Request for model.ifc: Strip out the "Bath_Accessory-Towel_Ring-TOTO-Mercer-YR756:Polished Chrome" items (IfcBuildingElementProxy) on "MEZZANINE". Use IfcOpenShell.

First a look at what the model holds.

```python
import ifcopenshell
import ifcopenshell.util.element

model = ifcopenshell.open("model.ifc")
print(model.schema)
storey = next(s for s in model.by_type("IfcBuildingStorey") if s.Name == "MEZZANINE")
proxies = [e for e in ifcopenshell.util.element.get_decomposition(storey) if e.is_a("IfcBuildingElementProxy")]
seen = {}
for e in proxies:
    element_type = ifcopenshell.util.element.get_type(e)
    name = element_type.Name if element_type not in (None, e) else None
    seen[name] = seen.get(name, 0) + 1
for name, count in sorted(seen.items(), key=str):
    print(count, "x", name)
```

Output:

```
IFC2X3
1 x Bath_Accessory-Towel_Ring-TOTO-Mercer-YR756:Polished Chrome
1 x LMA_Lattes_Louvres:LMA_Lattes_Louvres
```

```python
import ifcopenshell
import ifcopenshell.api.root
import ifcopenshell.util.element

model = ifcopenshell.open("model.ifc")

storey = next(s for s in model.by_type("IfcBuildingStorey") if s.Name == "MEZZANINE")
proxies = [e for e in ifcopenshell.util.element.get_decomposition(storey) if e.is_a("IfcBuildingElementProxy")]
targets = [e for e in proxies if (t := ifcopenshell.util.element.get_type(e)) not in (None, e) and t.Name == "Bath_Accessory-Towel_Ring-TOTO-Mercer-YR756:Polished Chrome"]

for e in targets:
    ifcopenshell.api.root.remove_product(model, product=e)
print(len(targets), "removed")

model.write("model_v2.ifc")
```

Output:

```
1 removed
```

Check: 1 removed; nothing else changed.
